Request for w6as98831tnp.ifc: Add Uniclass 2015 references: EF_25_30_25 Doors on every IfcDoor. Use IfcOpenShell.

First a look at what the model holds.

```python
import ifcopenshell

model = ifcopenshell.open("w6as98831tnp.ifc")
print(model.schema)
print("classifications:", [c.Name for c in model.by_type("IfcClassification")])
for ifc_class in ("IfcDoor", "IfcRoof", "IfcStair", "IfcWall", "IfcWindow"):
    print(ifc_class, len(model.by_type(ifc_class)))
```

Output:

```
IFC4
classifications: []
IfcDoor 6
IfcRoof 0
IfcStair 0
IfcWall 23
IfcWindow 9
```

```python
import ifcopenshell
import ifcopenshell.api.classification

model = ifcopenshell.open("w6as98831tnp.ifc")

system = ifcopenshell.api.classification.add_classification(model, classification="Uniclass 2015")

codes = {
    "IfcDoor": ("EF_25_30_25", "Doors"),
}
for ifc_class, (code, name) in codes.items():
    products = model.by_type(ifc_class)
    ifcopenshell.api.classification.add_reference(
        model, products=products, classification=system, identification=code, name=name
    )
    print(code, len(products))

model.write("w6as98831tnp_edited.ifc")
```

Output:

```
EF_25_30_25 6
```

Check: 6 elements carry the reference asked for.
